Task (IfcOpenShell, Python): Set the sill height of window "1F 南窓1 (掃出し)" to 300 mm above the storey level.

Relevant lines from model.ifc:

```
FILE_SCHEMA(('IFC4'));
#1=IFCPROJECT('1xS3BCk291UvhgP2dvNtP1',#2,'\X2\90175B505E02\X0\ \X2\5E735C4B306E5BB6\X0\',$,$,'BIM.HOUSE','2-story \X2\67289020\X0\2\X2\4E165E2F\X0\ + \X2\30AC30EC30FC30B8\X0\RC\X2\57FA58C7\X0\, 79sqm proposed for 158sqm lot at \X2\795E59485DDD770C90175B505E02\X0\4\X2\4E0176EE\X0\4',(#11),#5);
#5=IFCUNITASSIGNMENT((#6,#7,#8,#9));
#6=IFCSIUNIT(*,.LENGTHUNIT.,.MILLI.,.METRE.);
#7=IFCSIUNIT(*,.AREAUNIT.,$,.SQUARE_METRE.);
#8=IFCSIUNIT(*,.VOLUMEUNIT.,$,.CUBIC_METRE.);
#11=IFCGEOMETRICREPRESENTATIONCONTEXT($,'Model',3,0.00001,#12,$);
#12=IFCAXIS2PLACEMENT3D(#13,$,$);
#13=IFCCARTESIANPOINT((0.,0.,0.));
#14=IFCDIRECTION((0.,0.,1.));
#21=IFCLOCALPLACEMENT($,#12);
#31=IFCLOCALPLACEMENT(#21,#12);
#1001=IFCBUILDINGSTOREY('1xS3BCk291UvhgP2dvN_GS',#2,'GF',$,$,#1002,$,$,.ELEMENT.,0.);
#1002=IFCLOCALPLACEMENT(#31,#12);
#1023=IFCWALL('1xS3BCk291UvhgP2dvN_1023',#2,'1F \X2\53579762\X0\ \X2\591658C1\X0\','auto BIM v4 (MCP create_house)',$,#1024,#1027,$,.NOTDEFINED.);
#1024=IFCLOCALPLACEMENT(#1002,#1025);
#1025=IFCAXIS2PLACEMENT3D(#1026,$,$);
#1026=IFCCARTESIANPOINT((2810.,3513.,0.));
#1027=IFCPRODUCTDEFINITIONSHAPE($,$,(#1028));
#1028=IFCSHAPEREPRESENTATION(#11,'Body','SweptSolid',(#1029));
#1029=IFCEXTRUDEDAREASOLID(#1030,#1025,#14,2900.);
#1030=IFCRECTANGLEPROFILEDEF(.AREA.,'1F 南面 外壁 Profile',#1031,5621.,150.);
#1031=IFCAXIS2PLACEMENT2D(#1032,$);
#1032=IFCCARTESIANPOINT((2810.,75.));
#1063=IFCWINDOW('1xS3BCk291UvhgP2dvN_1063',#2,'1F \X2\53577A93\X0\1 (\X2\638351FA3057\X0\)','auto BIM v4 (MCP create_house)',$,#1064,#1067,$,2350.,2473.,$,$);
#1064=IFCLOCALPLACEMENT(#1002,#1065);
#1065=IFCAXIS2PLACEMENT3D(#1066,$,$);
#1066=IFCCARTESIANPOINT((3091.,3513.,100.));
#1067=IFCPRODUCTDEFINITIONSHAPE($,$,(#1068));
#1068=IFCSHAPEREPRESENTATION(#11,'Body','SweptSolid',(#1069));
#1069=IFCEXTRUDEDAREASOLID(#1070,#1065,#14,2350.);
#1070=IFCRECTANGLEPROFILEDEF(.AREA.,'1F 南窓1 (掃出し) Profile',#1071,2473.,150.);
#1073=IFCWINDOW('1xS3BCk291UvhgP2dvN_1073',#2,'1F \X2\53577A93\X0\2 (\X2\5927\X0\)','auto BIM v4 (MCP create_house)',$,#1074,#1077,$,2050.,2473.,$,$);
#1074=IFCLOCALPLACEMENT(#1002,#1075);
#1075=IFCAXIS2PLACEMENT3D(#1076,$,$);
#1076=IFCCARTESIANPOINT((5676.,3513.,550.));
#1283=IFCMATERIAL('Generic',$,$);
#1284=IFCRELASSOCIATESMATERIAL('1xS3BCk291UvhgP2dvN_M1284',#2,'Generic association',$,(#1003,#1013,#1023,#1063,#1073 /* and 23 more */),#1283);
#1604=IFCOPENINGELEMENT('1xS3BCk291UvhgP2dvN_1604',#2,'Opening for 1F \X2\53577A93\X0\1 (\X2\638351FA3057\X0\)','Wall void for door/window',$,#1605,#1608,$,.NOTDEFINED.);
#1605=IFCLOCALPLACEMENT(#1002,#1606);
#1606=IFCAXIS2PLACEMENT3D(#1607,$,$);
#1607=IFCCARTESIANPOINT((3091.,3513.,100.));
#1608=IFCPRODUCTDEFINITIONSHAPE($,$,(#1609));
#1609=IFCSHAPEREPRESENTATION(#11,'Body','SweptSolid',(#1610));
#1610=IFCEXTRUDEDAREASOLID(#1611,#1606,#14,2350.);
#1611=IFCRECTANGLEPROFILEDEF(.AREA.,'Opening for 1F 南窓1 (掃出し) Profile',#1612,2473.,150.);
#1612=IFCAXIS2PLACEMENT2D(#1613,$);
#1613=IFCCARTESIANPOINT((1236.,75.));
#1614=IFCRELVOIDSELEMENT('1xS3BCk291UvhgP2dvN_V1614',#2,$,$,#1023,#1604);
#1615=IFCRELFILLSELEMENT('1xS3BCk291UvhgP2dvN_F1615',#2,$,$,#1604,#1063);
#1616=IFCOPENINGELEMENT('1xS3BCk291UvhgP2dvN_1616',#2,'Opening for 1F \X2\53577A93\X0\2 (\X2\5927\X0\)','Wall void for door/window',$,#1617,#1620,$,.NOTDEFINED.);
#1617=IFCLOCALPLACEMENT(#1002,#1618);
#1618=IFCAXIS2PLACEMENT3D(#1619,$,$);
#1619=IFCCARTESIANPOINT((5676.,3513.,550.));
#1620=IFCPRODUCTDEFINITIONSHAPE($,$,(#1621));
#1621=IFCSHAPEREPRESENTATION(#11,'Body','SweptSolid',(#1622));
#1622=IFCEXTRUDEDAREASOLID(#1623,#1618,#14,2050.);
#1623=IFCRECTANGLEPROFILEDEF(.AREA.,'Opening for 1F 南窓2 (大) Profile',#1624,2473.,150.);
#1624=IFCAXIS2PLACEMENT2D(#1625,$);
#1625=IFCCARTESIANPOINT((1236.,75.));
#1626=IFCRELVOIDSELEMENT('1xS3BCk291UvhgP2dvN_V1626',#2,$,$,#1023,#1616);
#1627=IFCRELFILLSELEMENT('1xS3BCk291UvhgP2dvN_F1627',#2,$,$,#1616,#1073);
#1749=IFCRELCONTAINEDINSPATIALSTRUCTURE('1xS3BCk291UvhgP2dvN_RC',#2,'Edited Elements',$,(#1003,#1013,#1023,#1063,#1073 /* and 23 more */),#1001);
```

```python
import numpy as np
import ifcopenshell
import ifcopenshell.api.geometry
import ifcopenshell.geom
import ifcopenshell.util.element
import ifcopenshell.util.placement
import ifcopenshell.util.shape
import ifcopenshell.util.unit

model = ifcopenshell.open("model.ifc")
unit_scale = ifcopenshell.util.unit.calculate_unit_scale(model)

window = model.by_guid("1xS3BCk291UvhgP2dvN_1063")
opening = window.FillsVoids[0].RelatingOpeningElement
storey = ifcopenshell.util.element.get_container(window, ifc_class="IfcBuildingStorey")
level = ifcopenshell.util.placement.get_local_placement(storey.ObjectPlacement)[2, 3]

# The opening's origin need not be at the sill, so measure its lowest point.
shape = ifcopenshell.geom.create_shape(ifcopenshell.geom.settings(), opening)
bottom = ifcopenshell.util.shape.get_shape_bottom_elevation(shape, shape.geometry) / unit_scale
dz = level + 0.3 / unit_scale - bottom

shift = np.array([0.0, 0.0, dz])
# The window is not placed relative to its opening, so move both.
for product in (opening, window):
    matrix = ifcopenshell.util.placement.get_local_placement(product.ObjectPlacement)
    matrix[:3, 3] += shift
    ifcopenshell.api.geometry.edit_object_placement(model, product=product, matrix=matrix, is_si=False)

print(f"moved by {dz * unit_scale:+.3f} m")

model.write("model-out.ifc")
```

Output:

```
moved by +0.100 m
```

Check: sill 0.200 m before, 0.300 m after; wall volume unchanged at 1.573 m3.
